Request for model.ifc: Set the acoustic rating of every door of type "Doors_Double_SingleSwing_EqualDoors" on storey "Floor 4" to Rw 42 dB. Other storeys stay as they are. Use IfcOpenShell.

First a look at what the model holds.

```python
import ifcopenshell
import ifcopenshell.util.element

model = ifcopenshell.open("model.ifc")
print(model.schema)
storey = next(s for s in model.by_type("IfcBuildingStorey") if s.Name == "Floor 4")
doors = [e for e in ifcopenshell.util.element.get_decomposition(storey) if e.is_a("IfcDoor")]
seen = {}
for e in doors:
    element_type = ifcopenshell.util.element.get_type(e)
    key = (element_type.Name if element_type != e and element_type else None, ifcopenshell.util.element.get_pset(e, "Pset_DoorCommon", "AcousticRating"))
    seen[key] = seen.get(key, 0) + 1
for (name, value), count in sorted(seen.items(), key=str):
    print(count, "x", name, "|", value)
```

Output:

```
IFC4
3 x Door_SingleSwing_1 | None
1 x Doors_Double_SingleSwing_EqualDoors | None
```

```python
import ifcopenshell
import ifcopenshell.api.pset
import ifcopenshell.util.element

model = ifcopenshell.open("model.ifc")

storey = next(s for s in model.by_type("IfcBuildingStorey") if s.Name == "Floor 4")
doors = [e for e in ifcopenshell.util.element.get_decomposition(storey) if e.is_a("IfcDoor")]

count = 0
for e in doors:
    element_type = ifcopenshell.util.element.get_type(e)
    if element_type in (None, e) or element_type.Name != "Doors_Double_SingleSwing_EqualDoors":
        continue
    # add_pset returns the element's existing set when there is one.
    pset = ifcopenshell.api.pset.add_pset(model, product=e, name="Pset_DoorCommon")
    ifcopenshell.api.pset.edit_pset(model, pset=pset, properties={"AcousticRating": "Rw 42 dB"})
    count += 1

print(count, "doors updated")

model.write("model-out.ifc")
```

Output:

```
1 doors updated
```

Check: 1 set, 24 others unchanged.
